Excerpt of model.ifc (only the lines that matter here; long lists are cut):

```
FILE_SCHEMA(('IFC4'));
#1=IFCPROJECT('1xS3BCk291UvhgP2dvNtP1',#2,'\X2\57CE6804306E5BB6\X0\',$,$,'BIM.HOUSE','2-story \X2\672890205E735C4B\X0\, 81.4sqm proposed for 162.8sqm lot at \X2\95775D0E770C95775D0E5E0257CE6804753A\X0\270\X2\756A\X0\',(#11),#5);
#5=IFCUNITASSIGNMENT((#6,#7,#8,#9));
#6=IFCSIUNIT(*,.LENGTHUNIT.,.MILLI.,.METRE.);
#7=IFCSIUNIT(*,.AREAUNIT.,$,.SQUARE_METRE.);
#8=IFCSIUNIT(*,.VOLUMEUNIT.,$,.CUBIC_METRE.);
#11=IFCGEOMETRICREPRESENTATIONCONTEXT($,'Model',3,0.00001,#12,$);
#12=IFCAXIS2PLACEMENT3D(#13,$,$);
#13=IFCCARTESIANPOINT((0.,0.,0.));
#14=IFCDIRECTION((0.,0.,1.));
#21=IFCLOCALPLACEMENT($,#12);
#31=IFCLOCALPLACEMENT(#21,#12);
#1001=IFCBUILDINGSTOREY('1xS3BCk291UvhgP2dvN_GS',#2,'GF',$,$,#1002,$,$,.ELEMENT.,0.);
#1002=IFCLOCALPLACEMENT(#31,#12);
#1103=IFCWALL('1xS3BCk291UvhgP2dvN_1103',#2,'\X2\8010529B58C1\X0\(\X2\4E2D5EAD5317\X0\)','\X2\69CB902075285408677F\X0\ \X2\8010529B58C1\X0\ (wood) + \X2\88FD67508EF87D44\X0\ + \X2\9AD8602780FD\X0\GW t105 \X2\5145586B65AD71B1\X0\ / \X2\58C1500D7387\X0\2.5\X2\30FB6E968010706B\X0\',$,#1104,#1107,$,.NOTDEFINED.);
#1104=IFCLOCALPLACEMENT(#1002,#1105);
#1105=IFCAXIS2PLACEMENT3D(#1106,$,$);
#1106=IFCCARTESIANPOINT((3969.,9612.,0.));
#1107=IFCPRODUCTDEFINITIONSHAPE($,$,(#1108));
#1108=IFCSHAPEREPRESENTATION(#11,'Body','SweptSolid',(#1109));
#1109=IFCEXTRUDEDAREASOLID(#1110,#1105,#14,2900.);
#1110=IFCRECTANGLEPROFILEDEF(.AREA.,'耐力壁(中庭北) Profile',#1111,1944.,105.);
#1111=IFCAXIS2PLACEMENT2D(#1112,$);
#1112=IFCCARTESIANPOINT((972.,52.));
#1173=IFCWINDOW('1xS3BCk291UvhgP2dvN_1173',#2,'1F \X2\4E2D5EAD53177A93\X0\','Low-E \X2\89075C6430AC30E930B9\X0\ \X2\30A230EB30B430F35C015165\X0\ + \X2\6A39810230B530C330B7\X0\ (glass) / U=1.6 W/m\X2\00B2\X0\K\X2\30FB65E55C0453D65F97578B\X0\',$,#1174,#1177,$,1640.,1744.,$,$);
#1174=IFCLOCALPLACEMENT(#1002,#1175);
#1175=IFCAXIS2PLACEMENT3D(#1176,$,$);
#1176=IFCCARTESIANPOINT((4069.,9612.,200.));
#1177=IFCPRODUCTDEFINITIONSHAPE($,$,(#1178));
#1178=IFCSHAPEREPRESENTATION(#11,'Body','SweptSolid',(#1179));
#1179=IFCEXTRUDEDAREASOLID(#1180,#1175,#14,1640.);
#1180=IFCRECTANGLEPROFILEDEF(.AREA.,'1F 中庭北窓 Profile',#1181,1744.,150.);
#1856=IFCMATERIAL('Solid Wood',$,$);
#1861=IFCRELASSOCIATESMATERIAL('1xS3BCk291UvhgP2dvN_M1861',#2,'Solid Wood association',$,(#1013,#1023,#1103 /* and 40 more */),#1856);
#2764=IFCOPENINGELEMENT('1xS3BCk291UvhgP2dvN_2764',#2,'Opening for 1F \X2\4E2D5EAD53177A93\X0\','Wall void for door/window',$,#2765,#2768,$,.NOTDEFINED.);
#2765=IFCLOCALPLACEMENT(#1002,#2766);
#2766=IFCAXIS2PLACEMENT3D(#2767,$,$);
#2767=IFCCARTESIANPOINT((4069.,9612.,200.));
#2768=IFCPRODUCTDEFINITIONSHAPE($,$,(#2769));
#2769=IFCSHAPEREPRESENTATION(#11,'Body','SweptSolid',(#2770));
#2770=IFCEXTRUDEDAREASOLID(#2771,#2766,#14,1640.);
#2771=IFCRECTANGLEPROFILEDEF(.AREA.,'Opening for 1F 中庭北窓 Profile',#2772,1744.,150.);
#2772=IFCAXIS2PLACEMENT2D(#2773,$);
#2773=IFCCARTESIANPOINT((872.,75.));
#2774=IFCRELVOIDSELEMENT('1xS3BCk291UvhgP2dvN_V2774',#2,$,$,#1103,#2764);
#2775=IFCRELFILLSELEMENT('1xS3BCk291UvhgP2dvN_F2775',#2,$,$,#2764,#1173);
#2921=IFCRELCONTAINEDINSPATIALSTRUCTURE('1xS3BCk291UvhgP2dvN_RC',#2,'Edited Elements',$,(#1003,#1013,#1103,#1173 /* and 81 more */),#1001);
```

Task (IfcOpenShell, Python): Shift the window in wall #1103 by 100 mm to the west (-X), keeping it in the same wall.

```python
import ifcopenshell
import ifcopenshell.api.geometry
import ifcopenshell.util.placement
import ifcopenshell.util.unit

model = ifcopenshell.open("model.ifc")
unit_scale = ifcopenshell.util.unit.calculate_unit_scale(model)

window = model.by_guid("1xS3BCk291UvhgP2dvN_1173")
opening = window.FillsVoids[0].RelatingOpeningElement
wall = opening.VoidsElements[0].RelatingBuildingElement

wall_matrix = ifcopenshell.util.placement.get_local_placement(wall.ObjectPlacement)
shift = wall_matrix[:3, 0] * -0.1 / unit_scale
before = ifcopenshell.util.placement.get_local_placement(window.ObjectPlacement)[:3, 3].copy()

# The window is not placed relative to its opening, so move both.
for product in (opening, window):
    matrix = ifcopenshell.util.placement.get_local_placement(product.ObjectPlacement)
    matrix[:3, 3] += shift
    ifcopenshell.api.geometry.edit_object_placement(model, product=product, matrix=matrix, is_si=False)

after = ifcopenshell.util.placement.get_local_placement(window.ObjectPlacement)[:3, 3]
print("window moved by", (after - before).round(3) + 0.0)

model.write("model_updated.ifc")
```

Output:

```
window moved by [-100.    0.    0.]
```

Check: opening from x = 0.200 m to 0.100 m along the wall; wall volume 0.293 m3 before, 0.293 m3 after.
